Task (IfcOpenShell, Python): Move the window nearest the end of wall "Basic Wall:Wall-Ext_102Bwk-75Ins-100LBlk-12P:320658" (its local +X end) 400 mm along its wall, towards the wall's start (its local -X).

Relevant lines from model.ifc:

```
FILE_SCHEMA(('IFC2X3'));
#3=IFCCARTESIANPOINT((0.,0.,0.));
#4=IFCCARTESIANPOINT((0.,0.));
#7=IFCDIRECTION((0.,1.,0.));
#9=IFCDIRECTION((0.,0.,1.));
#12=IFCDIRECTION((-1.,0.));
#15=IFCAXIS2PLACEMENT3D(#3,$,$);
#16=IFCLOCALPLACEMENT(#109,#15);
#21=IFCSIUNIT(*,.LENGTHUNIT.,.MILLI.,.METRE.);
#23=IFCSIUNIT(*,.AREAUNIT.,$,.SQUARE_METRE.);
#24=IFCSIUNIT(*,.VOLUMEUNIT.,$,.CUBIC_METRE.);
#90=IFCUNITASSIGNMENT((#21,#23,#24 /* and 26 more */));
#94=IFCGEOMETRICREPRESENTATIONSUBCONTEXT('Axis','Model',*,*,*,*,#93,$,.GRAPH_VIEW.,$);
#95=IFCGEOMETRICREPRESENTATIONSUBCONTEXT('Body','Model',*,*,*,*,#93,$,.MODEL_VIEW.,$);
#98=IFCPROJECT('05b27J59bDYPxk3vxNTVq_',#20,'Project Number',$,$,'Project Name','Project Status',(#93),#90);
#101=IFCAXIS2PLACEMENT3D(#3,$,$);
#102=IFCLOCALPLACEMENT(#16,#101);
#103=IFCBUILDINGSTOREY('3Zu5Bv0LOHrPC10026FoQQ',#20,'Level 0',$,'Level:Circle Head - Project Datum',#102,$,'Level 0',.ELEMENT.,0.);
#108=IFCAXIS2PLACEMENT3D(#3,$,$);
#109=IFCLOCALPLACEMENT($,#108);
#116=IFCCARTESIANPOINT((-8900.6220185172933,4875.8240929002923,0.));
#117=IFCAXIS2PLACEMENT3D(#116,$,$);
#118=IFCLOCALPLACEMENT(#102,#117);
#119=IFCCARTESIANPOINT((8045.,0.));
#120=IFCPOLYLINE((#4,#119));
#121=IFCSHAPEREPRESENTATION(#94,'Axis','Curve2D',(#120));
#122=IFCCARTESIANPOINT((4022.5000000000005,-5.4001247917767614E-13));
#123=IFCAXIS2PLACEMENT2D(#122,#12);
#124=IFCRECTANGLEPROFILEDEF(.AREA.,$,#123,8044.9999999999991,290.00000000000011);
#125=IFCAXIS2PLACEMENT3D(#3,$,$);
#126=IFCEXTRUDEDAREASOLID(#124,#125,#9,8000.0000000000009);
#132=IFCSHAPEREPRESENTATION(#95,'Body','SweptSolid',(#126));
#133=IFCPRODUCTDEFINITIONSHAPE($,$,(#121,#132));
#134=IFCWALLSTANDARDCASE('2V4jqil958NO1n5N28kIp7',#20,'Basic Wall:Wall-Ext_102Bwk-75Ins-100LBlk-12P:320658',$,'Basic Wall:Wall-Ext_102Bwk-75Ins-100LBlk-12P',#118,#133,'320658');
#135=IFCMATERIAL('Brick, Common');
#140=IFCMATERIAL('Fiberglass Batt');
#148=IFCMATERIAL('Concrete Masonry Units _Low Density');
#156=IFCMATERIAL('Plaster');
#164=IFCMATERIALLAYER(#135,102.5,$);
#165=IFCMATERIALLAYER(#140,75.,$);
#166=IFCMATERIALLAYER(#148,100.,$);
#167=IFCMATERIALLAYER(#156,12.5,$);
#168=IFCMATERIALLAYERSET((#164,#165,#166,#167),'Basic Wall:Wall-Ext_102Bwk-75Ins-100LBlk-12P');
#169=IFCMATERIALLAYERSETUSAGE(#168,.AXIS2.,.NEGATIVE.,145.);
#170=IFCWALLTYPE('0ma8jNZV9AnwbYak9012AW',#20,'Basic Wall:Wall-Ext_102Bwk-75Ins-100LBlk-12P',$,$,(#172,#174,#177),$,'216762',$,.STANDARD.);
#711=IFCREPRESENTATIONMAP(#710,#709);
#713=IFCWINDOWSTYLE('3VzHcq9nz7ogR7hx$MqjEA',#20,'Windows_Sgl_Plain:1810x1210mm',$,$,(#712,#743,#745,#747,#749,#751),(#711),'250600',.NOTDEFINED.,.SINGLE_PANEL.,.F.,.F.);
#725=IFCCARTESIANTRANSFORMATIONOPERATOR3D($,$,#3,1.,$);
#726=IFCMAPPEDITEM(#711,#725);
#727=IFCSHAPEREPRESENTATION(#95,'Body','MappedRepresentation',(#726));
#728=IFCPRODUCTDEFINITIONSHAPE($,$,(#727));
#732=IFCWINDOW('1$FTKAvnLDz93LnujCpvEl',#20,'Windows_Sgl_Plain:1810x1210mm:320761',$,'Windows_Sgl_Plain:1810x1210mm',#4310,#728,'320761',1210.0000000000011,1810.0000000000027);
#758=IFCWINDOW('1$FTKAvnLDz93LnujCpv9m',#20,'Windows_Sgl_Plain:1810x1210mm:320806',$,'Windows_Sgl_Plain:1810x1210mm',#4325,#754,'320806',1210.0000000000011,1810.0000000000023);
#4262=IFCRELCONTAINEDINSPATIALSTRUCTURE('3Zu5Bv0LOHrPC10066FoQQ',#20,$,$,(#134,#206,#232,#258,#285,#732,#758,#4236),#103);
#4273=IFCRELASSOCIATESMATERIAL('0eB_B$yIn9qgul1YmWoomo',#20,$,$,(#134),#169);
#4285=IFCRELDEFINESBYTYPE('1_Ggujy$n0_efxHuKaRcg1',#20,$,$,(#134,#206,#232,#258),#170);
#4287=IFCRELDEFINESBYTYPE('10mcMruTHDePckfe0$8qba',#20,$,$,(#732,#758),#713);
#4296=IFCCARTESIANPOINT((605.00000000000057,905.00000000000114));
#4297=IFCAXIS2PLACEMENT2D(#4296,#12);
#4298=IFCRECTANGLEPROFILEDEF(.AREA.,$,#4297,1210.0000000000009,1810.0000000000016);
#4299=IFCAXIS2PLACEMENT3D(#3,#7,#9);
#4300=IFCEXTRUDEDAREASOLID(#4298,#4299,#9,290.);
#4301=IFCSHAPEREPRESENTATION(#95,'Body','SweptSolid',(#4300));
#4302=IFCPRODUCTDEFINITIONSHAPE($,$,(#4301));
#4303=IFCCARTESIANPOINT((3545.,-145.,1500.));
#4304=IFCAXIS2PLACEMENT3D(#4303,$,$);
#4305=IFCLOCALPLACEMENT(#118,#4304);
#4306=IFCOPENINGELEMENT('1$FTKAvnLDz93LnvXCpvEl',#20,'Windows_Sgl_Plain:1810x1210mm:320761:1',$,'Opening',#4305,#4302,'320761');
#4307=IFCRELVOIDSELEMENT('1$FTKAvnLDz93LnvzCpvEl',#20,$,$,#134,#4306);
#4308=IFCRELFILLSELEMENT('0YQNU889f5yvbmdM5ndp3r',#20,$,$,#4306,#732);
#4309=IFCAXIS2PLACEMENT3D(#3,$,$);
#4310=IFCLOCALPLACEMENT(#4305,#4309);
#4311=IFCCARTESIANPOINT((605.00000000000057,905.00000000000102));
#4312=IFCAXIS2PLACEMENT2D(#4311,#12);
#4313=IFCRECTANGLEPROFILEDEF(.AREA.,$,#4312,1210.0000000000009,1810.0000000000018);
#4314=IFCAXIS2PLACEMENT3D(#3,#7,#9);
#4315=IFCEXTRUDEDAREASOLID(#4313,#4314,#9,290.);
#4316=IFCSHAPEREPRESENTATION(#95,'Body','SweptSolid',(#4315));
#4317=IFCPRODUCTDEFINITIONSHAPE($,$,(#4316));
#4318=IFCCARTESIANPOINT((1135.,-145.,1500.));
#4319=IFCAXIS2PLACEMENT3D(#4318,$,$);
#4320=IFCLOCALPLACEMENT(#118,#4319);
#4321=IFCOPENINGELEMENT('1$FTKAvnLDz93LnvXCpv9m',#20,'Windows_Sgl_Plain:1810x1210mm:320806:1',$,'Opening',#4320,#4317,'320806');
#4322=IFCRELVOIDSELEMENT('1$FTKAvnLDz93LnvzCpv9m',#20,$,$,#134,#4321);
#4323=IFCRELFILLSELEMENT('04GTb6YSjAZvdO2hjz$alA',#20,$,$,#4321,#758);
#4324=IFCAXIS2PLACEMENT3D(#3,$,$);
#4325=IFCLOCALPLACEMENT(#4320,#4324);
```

```python
import ifcopenshell
import ifcopenshell.api.geometry
import ifcopenshell.util.placement
import ifcopenshell.util.unit

model = ifcopenshell.open("model.ifc")
unit_scale = ifcopenshell.util.unit.calculate_unit_scale(model)

window = model.by_guid("1$FTKAvnLDz93LnujCpvEl")
opening = window.FillsVoids[0].RelatingOpeningElement
wall = opening.VoidsElements[0].RelatingBuildingElement

wall_matrix = ifcopenshell.util.placement.get_local_placement(wall.ObjectPlacement)
shift = wall_matrix[:3, 0] * -0.4 / unit_scale
before = ifcopenshell.util.placement.get_local_placement(window.ObjectPlacement)[:3, 3].copy()

# The window is placed relative to its opening, so it follows when the opening moves.
matrix = ifcopenshell.util.placement.get_local_placement(opening.ObjectPlacement)
matrix[:3, 3] += shift
ifcopenshell.api.geometry.edit_object_placement(
    model, product=opening, matrix=matrix, is_si=False, should_transform_children=True
)

after = ifcopenshell.util.placement.get_local_placement(window.ObjectPlacement)[:3, 3]
print("window moved by", (after - before).round(3) + 0.0)

model.write("model_edited.ifc")
```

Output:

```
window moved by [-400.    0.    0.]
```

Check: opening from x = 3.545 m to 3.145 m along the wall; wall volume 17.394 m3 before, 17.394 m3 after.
